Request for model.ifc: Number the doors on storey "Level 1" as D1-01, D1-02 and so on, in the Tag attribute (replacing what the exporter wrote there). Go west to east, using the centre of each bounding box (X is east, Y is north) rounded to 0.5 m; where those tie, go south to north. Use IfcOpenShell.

First a look at what the model holds.

```python
import ifcopenshell
import ifcopenshell.util.element
import ifcopenshell.util.placement

model = ifcopenshell.open("model.ifc")
print(model.schema)
storey = next(s for s in model.by_type("IfcBuildingStorey") if s.Name == "Level 1")
doors = [e for e in ifcopenshell.util.element.get_decomposition(storey) if e.is_a("IfcDoor")]
for e in sorted(doors, key=lambda e: e.id()):
    origin = ifcopenshell.util.placement.get_local_placement(e.ObjectPlacement)[:3, 3]
    print(e.id(), e.Tag, e.Name, origin.round(2) + 0.0, sep=" | ")
```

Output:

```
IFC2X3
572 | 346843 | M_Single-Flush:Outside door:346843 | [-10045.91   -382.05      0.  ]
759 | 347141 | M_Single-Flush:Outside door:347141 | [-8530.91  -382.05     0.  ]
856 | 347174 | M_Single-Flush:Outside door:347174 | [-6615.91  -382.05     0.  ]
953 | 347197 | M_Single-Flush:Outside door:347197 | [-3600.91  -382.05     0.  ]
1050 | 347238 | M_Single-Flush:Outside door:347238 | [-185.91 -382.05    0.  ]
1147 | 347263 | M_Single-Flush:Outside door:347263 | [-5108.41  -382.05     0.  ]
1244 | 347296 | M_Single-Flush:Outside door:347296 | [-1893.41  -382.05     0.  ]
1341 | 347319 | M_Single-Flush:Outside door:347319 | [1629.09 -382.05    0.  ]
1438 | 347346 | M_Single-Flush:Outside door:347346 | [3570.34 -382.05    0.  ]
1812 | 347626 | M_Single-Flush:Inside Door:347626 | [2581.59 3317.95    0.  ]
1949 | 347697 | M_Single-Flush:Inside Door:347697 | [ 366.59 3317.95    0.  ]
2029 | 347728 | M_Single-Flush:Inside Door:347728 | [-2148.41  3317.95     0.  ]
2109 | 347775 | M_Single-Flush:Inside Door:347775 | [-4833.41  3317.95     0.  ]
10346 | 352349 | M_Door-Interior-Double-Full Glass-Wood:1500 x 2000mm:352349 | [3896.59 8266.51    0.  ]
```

```python
import ifcopenshell
import ifcopenshell.geom
import ifcopenshell.util.element
import ifcopenshell.util.shape

model = ifcopenshell.open("model.ifc")
settings = ifcopenshell.geom.settings()
settings.set("use-world-coords", True)


def centre(element):
    shape = ifcopenshell.geom.create_shape(settings, element)
    return ifcopenshell.util.shape.get_bbox_centroid(shape.geometry)


storey = next(s for s in model.by_type("IfcBuildingStorey") if s.Name == "Level 1")
doors = [e for e in ifcopenshell.util.element.get_decomposition(storey) if e.is_a("IfcDoor")]

# Insertion points can sit at a corner or the storey origin, so sort by the geometry (in metres).
centres = {e: centre(e) for e in doors}
doors.sort(key=lambda e: (round(centres[e][0] / 0.5), centres[e][1]))

for i, e in enumerate(doors, start=1):
    number = f"D1-{i:02d}"
    e.Tag = number
    print(e.id(), number)

model.write("model_updated.ifc")
```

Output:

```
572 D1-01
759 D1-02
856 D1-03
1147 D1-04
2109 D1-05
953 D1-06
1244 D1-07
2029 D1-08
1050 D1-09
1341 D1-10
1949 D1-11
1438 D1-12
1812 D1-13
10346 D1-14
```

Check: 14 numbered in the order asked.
